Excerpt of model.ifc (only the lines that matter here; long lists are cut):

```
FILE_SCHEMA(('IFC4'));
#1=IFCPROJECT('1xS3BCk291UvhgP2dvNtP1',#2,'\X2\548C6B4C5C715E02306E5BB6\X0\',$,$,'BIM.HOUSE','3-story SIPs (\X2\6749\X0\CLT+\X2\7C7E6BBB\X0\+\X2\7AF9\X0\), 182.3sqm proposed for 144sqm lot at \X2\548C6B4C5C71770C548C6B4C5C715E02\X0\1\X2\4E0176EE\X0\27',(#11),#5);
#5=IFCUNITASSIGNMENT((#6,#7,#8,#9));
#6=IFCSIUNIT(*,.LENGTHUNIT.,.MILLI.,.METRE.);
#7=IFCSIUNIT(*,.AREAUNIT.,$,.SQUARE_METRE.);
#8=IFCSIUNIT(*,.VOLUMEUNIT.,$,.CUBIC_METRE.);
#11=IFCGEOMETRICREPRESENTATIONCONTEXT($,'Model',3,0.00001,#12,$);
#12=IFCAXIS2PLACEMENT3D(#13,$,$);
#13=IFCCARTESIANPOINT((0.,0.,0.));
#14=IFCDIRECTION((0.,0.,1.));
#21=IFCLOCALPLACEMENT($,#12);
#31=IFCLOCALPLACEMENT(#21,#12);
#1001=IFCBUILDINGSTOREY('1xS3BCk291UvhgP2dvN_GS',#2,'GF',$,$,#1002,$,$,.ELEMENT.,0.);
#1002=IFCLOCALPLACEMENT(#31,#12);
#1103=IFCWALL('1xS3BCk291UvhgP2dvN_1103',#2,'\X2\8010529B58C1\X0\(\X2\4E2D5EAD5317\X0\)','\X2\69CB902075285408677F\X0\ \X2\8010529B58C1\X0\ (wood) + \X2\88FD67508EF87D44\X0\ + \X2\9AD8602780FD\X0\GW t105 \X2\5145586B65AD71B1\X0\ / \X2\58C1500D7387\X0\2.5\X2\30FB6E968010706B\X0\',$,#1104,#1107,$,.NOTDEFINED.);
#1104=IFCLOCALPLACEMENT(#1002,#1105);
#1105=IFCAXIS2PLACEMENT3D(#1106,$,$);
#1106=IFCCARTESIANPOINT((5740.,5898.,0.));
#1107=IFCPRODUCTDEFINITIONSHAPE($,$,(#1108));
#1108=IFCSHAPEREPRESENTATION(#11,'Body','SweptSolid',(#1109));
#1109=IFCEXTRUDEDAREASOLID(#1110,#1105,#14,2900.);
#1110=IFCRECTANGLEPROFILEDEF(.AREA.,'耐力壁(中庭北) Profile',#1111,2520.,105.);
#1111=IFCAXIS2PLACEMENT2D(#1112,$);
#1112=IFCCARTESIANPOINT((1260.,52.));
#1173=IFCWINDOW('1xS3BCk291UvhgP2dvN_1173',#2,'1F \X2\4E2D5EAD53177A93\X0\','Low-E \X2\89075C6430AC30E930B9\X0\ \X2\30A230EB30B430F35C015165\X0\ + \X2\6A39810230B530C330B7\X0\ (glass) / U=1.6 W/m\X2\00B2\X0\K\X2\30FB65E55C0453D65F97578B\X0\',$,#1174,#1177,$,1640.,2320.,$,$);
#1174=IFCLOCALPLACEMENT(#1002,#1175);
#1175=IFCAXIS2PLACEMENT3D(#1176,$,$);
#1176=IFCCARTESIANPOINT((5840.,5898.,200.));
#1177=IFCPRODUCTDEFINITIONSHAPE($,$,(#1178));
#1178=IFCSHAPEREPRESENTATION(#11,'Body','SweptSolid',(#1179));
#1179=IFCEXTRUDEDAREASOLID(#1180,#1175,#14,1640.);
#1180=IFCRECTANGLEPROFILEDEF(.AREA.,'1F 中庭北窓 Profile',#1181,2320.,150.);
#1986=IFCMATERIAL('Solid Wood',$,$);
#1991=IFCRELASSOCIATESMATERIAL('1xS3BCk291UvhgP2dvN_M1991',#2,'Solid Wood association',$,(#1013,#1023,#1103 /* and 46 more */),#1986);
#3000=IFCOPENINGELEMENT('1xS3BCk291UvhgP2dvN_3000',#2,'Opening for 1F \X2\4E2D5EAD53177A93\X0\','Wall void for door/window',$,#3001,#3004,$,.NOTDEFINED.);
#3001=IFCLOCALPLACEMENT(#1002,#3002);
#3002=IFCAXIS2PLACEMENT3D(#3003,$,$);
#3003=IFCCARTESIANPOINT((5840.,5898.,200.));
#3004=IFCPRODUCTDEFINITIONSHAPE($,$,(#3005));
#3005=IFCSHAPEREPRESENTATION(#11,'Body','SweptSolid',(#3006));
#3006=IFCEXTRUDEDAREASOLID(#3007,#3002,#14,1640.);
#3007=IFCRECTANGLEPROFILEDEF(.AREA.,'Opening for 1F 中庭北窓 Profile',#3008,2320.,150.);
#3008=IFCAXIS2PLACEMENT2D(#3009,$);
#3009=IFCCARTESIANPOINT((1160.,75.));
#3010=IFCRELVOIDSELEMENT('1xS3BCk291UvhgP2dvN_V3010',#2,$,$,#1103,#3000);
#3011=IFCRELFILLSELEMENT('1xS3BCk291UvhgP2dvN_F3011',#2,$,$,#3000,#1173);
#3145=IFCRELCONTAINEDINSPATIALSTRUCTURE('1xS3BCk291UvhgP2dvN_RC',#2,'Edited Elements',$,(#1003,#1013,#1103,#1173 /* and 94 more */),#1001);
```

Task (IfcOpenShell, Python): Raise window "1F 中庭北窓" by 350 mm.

```python
import numpy as np
import ifcopenshell
import ifcopenshell.api.geometry
import ifcopenshell.util.placement
import ifcopenshell.util.unit

model = ifcopenshell.open("model.ifc")
unit_scale = ifcopenshell.util.unit.calculate_unit_scale(model)

window = model.by_guid("1xS3BCk291UvhgP2dvN_1173")
opening = window.FillsVoids[0].RelatingOpeningElement
dz = 350.0

shift = np.array([0.0, 0.0, dz])
# The window is not placed relative to its opening, so move both.
for product in (opening, window):
    matrix = ifcopenshell.util.placement.get_local_placement(product.ObjectPlacement)
    matrix[:3, 3] += shift
    ifcopenshell.api.geometry.edit_object_placement(model, product=product, matrix=matrix, is_si=False)

print(f"moved by {dz * unit_scale:+.3f} m")

model.write("model_v2.ifc")
```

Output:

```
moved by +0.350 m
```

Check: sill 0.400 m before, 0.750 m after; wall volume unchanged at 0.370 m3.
